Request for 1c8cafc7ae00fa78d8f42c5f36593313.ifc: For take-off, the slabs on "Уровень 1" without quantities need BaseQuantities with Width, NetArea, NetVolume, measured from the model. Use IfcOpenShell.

First a look at what the model holds.

```python
import ifcopenshell
import ifcopenshell.util.element
import ifcopenshell.util.unit

model = ifcopenshell.open("1c8cafc7ae00fa78d8f42c5f36593313.ifc")
print(model.schema)
for unit_type in ("LENGTHUNIT", "AREAUNIT", "VOLUMEUNIT"):
    print(unit_type, ifcopenshell.util.unit.calculate_unit_scale(model, unit_type))
storey = next(s for s in model.by_type("IfcBuildingStorey") if s.Name == "Уровень 1")
slabs = [e for e in ifcopenshell.util.element.get_decomposition(storey) if e.is_a("IfcSlab")]
for e in sorted(slabs, key=lambda e: e.id()):
    print(e.id(), e.is_a(), e.Name, list(ifcopenshell.util.element.get_psets(e, qtos_only=True)), sep=" | ")
```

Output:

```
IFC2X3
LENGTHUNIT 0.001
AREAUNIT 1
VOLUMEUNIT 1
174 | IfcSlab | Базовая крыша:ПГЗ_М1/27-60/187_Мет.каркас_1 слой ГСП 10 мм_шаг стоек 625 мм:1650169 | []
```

```python
import ifcopenshell
import ifcopenshell.api.pset
import ifcopenshell.geom
import ifcopenshell.util.element
import ifcopenshell.util.shape
import ifcopenshell.util.unit

model = ifcopenshell.open("1c8cafc7ae00fa78d8f42c5f36593313.ifc")
unit_scale = ifcopenshell.util.unit.calculate_unit_scale(model)
area_scale = ifcopenshell.util.unit.calculate_unit_scale(model, "AREAUNIT")
volume_scale = ifcopenshell.util.unit.calculate_unit_scale(model, "VOLUMEUNIT")
settings = ifcopenshell.geom.settings()

storey = next(s for s in model.by_type("IfcBuildingStorey") if s.Name == "Уровень 1")
slabs = [e for e in ifcopenshell.util.element.get_decomposition(storey) if e.is_a("IfcSlab")]

for e in sorted(slabs, key=lambda e: e.id()):
    if ifcopenshell.util.element.get_psets(e, qtos_only=True, should_inherit=False):
        continue
    # Geometry comes back in metres, in the element's own axes.
    shape = ifcopenshell.geom.create_shape(settings, e)
    values = {
        "Width": ifcopenshell.util.shape.get_z(shape.geometry) / unit_scale,
        "NetArea": ifcopenshell.util.shape.get_footprint_area(shape.geometry) / area_scale,
        "NetVolume": ifcopenshell.util.shape.get_volume(shape.geometry) / volume_scale,
    }
    qto = ifcopenshell.api.pset.add_qto(model, product=e, name="BaseQuantities")
    ifcopenshell.api.pset.edit_qto(model, qto=qto, properties=values)
    print(e.id(), {k: round(v, 3) for k, v in values.items()})

model.write("1c8cafc7ae00fa78d8f42c5f36593313_edited.ifc")
```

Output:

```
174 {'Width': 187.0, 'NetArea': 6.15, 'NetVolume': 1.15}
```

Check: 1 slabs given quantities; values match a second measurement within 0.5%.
